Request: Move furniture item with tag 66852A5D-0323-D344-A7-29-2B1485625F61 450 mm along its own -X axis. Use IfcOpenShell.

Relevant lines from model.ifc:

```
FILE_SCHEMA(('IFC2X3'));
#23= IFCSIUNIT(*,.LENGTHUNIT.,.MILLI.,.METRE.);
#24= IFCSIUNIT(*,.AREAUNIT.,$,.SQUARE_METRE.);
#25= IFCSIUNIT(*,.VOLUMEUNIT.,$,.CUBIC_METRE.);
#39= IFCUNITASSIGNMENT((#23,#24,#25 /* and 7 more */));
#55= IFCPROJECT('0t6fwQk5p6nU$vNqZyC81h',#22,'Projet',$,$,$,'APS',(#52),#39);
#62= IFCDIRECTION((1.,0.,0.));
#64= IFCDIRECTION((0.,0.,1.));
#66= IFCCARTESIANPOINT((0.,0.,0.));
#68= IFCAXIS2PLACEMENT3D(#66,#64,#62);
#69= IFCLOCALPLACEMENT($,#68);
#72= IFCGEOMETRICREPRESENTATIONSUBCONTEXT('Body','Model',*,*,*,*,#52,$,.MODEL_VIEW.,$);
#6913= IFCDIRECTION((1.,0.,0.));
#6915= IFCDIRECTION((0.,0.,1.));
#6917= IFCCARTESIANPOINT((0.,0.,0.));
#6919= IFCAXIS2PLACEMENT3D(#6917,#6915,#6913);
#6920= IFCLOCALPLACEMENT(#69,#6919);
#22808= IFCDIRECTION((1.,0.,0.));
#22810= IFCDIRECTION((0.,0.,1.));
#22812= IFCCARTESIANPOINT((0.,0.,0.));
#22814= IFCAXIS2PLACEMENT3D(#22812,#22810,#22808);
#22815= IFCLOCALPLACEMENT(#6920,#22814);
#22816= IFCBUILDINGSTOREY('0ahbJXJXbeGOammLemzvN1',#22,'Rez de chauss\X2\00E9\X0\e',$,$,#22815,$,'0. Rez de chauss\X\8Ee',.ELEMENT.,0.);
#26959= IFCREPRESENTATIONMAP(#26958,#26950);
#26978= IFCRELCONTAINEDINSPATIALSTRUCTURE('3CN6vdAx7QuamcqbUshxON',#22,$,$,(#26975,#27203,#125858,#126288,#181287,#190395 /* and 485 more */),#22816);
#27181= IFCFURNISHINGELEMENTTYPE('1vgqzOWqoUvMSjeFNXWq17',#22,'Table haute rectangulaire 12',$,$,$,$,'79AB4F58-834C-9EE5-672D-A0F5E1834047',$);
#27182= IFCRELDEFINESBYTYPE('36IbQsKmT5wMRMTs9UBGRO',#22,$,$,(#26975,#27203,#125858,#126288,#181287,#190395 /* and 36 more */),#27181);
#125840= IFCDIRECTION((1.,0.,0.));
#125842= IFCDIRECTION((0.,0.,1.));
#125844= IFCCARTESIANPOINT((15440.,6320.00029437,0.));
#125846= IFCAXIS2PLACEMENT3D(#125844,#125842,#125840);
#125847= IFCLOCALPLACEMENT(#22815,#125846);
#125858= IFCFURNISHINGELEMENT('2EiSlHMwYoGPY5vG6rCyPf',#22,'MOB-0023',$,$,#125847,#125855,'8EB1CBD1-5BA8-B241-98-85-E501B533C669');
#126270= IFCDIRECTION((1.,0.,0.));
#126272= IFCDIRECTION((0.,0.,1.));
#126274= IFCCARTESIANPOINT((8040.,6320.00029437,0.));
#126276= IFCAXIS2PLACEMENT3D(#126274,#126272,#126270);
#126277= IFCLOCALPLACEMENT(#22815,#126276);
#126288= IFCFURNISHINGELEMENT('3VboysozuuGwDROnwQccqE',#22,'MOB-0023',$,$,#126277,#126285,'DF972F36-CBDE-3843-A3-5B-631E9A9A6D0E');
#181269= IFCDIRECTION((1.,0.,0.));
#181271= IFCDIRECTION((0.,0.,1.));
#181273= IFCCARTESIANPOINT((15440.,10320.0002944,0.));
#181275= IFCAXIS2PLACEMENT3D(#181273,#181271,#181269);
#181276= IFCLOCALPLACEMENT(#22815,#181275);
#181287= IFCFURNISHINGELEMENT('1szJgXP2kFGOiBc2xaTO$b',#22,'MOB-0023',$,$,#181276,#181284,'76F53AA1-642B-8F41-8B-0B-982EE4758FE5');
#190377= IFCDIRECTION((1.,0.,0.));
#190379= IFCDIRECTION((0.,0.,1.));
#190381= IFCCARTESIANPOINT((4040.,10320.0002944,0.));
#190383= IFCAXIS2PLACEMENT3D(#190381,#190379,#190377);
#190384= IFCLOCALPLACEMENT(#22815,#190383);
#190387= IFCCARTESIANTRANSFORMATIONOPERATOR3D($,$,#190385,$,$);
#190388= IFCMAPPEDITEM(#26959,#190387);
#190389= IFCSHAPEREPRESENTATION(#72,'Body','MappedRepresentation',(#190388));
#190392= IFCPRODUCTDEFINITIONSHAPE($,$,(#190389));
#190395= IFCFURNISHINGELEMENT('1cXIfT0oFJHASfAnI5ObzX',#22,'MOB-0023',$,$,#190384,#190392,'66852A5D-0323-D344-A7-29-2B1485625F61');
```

```python
import ifcopenshell
import ifcopenshell.api.geometry
import ifcopenshell.util.placement

model = ifcopenshell.open("model.ifc")

item = model.by_guid("1cXIfT0oFJHASfAnI5ObzX")
matrix = ifcopenshell.util.placement.get_local_placement(item.ObjectPlacement)
matrix[:3, 3] -= matrix[:3, 0] * 450.0
ifcopenshell.api.geometry.edit_object_placement(model, product=item, matrix=matrix, is_si=False)

print(ifcopenshell.util.placement.get_local_placement(item.ObjectPlacement).round(3) + 0.0)

model.write("model-out.ifc")
```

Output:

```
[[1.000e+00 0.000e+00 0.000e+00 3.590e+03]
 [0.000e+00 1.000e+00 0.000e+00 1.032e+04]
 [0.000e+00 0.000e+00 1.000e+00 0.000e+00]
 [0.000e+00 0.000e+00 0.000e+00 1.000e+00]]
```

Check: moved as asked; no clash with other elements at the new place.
